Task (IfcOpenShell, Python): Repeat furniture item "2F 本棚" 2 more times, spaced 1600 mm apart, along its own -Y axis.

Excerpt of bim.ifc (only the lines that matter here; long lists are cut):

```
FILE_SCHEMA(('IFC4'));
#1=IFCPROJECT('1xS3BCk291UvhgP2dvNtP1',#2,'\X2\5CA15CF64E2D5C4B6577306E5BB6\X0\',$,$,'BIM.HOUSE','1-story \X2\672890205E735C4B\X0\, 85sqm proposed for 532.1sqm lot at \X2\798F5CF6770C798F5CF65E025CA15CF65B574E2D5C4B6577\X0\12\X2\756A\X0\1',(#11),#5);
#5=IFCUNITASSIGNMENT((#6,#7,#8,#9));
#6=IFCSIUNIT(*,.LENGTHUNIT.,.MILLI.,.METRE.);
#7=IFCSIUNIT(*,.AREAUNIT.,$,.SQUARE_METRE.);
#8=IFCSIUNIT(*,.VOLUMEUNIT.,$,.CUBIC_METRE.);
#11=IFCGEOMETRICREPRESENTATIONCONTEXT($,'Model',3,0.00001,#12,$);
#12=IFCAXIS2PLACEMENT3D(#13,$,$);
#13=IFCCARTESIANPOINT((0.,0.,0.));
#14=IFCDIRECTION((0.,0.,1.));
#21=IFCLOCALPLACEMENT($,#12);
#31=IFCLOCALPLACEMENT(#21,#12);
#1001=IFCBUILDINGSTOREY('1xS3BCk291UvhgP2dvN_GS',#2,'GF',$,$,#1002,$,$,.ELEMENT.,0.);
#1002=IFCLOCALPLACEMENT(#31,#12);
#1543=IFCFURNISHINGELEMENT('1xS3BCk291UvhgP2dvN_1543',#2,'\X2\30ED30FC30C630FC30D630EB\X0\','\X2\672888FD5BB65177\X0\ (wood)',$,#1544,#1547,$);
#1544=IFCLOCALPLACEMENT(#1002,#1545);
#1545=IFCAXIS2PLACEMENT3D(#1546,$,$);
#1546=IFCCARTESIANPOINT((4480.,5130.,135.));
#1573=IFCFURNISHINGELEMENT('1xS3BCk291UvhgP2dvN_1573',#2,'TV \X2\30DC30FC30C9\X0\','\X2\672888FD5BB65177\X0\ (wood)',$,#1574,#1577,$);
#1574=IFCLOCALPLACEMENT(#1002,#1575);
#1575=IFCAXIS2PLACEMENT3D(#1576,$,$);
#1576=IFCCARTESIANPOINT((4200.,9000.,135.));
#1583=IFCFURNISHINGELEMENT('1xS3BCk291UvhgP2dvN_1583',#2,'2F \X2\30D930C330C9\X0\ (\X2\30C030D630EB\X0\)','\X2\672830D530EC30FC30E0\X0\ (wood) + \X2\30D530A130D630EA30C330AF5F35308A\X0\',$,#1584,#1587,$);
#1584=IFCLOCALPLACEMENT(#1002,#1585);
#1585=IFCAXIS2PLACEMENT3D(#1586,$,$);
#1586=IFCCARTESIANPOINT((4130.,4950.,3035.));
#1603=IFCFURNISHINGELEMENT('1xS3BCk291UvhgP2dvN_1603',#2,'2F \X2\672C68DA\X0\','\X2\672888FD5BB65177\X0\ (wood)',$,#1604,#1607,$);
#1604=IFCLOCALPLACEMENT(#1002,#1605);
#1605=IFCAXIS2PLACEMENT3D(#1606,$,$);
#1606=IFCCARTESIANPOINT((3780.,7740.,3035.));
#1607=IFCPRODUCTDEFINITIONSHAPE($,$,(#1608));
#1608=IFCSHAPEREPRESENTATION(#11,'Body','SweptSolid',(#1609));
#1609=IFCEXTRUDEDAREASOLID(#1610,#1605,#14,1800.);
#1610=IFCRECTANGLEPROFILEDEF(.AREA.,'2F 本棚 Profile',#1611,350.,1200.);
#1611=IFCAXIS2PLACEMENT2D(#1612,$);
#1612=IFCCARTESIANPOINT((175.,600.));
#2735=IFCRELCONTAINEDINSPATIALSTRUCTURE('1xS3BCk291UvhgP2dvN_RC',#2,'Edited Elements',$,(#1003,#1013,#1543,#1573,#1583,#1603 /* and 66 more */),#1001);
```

```python
import ifcopenshell
import ifcopenshell.api.geometry
import ifcopenshell.api.root
import ifcopenshell.util.element
import ifcopenshell.util.placement
import ifcopenshell.util.unit

model = ifcopenshell.open("bim.ifc")
unit_scale = ifcopenshell.util.unit.calculate_unit_scale(model)


def reuse_history(source, copy):
    """copy_class also copies each property set's owner history, people and application; keep the originals."""
    for rel in copy.IsDefinedBy:
        if rel.is_a("IfcRelDefinesByProperties") and (history := rel.RelatingPropertyDefinition.OwnerHistory):
            rel.RelatingPropertyDefinition.OwnerHistory = source.OwnerHistory
            ifcopenshell.util.element.remove_deep2(model, history)


source = model.by_guid("1xS3BCk291UvhgP2dvN_1603")
base = ifcopenshell.util.placement.get_local_placement(source.ObjectPlacement)
step = -base[:3, 1] * 1.6 / unit_scale

for i in range(1, 3):
    copy = ifcopenshell.api.root.copy_class(model, product=source)
    copy.Representation = ifcopenshell.util.element.copy_deep(
        model, source.Representation, exclude=["IfcGeometricRepresentationContext", "IfcRepresentationMap"]
    )
    reuse_history(source, copy)
    matrix = base.copy()
    matrix[:3, 3] += i * step
    print("added at", matrix[:3, 3].round(3) + 0.0)
    ifcopenshell.api.geometry.edit_object_placement(model, product=copy, matrix=matrix, is_si=False)

model.write("bim_rev.ifc")
```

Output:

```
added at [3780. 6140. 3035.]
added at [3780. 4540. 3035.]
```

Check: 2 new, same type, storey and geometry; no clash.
